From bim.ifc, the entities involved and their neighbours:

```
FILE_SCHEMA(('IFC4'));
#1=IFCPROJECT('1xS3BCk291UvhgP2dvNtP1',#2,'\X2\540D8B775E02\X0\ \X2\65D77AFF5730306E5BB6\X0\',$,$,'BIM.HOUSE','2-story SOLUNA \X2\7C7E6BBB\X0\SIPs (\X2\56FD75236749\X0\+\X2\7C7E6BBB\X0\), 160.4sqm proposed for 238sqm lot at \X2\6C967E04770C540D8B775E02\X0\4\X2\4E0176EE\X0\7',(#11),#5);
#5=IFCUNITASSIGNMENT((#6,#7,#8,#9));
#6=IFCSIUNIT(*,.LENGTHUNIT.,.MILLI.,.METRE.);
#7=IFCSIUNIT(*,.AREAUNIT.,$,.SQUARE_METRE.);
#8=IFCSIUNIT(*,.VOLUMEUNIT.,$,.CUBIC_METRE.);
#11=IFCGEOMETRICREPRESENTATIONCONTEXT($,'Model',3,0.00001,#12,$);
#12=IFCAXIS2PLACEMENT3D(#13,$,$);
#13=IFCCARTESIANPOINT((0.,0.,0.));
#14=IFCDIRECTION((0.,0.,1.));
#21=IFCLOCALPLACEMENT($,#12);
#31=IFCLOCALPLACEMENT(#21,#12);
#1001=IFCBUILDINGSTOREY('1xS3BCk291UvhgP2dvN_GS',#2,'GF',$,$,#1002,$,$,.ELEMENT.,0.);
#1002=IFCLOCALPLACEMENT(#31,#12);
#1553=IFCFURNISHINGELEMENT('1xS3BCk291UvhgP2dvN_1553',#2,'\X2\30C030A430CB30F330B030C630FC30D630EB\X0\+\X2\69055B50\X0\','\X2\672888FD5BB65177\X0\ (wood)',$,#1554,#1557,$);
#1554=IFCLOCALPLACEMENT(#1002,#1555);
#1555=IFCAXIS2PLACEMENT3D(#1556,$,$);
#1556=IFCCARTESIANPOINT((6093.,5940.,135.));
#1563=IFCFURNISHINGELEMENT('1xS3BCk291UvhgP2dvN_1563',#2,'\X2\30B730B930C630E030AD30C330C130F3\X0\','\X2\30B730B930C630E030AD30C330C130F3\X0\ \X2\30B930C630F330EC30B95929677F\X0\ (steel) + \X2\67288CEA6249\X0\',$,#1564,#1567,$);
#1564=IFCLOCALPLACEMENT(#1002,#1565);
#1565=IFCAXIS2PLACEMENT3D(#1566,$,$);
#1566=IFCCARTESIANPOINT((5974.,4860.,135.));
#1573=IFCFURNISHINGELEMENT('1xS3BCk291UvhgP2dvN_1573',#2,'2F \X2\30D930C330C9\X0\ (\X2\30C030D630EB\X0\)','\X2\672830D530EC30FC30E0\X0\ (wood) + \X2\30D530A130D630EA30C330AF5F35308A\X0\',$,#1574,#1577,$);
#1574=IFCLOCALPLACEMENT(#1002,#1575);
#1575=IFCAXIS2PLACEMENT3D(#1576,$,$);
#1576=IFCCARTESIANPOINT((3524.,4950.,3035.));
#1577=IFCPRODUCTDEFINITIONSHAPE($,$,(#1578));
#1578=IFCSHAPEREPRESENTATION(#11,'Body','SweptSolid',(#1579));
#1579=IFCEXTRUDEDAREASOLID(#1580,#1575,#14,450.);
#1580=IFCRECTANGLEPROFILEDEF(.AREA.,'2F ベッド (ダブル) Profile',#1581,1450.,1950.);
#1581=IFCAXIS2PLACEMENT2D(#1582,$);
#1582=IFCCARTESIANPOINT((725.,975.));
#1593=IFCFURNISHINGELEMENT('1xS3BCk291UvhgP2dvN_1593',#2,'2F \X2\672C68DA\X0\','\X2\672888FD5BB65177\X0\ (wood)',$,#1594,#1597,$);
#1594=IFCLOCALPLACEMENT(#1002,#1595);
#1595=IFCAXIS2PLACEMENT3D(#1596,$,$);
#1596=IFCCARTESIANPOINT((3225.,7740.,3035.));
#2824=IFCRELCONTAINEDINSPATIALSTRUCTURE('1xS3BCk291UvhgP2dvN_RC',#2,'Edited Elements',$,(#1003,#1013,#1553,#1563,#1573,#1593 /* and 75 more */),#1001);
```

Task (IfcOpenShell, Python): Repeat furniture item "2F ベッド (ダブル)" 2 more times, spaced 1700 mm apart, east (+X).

```python
import numpy as np
import ifcopenshell
import ifcopenshell.api.geometry
import ifcopenshell.api.root
import ifcopenshell.util.element
import ifcopenshell.util.placement

model = ifcopenshell.open("bim.ifc")


def reuse_history(source, copy):
    """copy_class also copies each property set's owner history, people and application; keep the originals."""
    for rel in copy.IsDefinedBy:
        if rel.is_a("IfcRelDefinesByProperties") and (history := rel.RelatingPropertyDefinition.OwnerHistory):
            rel.RelatingPropertyDefinition.OwnerHistory = source.OwnerHistory
            ifcopenshell.util.element.remove_deep2(model, history)


source = model.by_guid("1xS3BCk291UvhgP2dvN_1573")
base = ifcopenshell.util.placement.get_local_placement(source.ObjectPlacement)
step = np.array([1.0, 0.0, 0.0]) * 1700.0

for i in range(1, 3):
    copy = ifcopenshell.api.root.copy_class(model, product=source)
    copy.Representation = ifcopenshell.util.element.copy_deep(
        model, source.Representation, exclude=["IfcGeometricRepresentationContext", "IfcRepresentationMap"]
    )
    reuse_history(source, copy)
    matrix = base.copy()
    matrix[:3, 3] += i * step
    print("added at", matrix[:3, 3].round(3) + 0.0)
    ifcopenshell.api.geometry.edit_object_placement(model, product=copy, matrix=matrix, is_si=False)

model.write("bim_rev.ifc")
```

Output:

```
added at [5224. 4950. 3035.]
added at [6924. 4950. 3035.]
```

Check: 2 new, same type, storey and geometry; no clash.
